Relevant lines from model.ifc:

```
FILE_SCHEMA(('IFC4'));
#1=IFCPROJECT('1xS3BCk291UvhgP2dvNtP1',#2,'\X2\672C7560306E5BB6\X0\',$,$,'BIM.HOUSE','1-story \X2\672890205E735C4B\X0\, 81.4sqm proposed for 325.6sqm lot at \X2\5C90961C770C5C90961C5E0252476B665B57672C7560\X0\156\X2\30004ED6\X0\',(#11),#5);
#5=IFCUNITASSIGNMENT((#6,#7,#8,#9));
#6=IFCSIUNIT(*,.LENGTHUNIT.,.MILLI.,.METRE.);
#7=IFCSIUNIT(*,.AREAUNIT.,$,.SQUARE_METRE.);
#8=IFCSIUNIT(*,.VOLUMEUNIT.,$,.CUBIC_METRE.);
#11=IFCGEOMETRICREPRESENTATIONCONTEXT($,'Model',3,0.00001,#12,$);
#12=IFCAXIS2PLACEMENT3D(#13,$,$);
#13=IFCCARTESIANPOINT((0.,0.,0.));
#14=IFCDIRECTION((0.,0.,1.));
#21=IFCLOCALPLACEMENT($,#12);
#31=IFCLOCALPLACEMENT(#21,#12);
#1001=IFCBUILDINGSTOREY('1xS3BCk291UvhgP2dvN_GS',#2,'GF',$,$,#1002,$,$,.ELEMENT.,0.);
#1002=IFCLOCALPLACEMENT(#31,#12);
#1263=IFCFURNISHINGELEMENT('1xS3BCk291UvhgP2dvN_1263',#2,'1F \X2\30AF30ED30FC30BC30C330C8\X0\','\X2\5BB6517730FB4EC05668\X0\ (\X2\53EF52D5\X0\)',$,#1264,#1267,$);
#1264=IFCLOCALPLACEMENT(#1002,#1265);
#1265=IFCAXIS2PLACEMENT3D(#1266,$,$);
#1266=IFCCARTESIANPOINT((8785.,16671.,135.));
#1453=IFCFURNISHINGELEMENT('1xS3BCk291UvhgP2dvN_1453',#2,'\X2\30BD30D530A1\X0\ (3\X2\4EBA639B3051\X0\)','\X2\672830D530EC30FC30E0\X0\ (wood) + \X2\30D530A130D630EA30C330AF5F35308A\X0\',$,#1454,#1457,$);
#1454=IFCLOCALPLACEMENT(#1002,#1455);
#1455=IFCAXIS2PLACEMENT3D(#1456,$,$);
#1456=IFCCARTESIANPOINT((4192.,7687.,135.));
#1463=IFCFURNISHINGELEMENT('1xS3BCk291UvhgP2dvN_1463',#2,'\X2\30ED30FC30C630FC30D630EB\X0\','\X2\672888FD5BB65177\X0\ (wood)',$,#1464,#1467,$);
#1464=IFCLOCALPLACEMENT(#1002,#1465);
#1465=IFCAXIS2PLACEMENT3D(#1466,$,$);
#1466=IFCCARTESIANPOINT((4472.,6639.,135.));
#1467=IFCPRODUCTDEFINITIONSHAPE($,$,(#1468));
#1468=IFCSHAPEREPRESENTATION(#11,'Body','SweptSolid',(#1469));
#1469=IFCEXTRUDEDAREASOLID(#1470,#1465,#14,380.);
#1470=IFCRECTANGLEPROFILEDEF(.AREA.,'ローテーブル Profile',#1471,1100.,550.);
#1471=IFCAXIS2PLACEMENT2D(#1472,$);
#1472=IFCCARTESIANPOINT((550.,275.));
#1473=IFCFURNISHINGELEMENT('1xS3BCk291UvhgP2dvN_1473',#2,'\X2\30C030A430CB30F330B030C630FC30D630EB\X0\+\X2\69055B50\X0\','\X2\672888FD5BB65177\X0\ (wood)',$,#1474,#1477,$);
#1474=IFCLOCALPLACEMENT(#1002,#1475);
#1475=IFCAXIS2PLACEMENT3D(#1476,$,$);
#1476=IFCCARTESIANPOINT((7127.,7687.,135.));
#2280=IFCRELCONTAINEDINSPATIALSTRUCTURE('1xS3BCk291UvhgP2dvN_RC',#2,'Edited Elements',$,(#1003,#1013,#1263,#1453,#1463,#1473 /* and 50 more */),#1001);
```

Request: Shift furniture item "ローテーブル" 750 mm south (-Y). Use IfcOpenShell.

```python
import ifcopenshell
import ifcopenshell.api.geometry
import ifcopenshell.util.placement
import ifcopenshell.util.unit

model = ifcopenshell.open("model.ifc")
unit_scale = ifcopenshell.util.unit.calculate_unit_scale(model)

item = model.by_guid("1xS3BCk291UvhgP2dvN_1463")
matrix = ifcopenshell.util.placement.get_local_placement(item.ObjectPlacement)
matrix[1, 3] -= 0.75 / unit_scale
ifcopenshell.api.geometry.edit_object_placement(model, product=item, matrix=matrix, is_si=False)

print(ifcopenshell.util.placement.get_local_placement(item.ObjectPlacement).round(3) + 0.0)

model.write("model_updated.ifc")
```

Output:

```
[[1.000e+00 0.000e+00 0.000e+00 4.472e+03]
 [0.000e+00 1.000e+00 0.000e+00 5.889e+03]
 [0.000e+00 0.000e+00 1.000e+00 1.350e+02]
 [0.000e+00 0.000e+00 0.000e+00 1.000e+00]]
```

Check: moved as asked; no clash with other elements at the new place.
